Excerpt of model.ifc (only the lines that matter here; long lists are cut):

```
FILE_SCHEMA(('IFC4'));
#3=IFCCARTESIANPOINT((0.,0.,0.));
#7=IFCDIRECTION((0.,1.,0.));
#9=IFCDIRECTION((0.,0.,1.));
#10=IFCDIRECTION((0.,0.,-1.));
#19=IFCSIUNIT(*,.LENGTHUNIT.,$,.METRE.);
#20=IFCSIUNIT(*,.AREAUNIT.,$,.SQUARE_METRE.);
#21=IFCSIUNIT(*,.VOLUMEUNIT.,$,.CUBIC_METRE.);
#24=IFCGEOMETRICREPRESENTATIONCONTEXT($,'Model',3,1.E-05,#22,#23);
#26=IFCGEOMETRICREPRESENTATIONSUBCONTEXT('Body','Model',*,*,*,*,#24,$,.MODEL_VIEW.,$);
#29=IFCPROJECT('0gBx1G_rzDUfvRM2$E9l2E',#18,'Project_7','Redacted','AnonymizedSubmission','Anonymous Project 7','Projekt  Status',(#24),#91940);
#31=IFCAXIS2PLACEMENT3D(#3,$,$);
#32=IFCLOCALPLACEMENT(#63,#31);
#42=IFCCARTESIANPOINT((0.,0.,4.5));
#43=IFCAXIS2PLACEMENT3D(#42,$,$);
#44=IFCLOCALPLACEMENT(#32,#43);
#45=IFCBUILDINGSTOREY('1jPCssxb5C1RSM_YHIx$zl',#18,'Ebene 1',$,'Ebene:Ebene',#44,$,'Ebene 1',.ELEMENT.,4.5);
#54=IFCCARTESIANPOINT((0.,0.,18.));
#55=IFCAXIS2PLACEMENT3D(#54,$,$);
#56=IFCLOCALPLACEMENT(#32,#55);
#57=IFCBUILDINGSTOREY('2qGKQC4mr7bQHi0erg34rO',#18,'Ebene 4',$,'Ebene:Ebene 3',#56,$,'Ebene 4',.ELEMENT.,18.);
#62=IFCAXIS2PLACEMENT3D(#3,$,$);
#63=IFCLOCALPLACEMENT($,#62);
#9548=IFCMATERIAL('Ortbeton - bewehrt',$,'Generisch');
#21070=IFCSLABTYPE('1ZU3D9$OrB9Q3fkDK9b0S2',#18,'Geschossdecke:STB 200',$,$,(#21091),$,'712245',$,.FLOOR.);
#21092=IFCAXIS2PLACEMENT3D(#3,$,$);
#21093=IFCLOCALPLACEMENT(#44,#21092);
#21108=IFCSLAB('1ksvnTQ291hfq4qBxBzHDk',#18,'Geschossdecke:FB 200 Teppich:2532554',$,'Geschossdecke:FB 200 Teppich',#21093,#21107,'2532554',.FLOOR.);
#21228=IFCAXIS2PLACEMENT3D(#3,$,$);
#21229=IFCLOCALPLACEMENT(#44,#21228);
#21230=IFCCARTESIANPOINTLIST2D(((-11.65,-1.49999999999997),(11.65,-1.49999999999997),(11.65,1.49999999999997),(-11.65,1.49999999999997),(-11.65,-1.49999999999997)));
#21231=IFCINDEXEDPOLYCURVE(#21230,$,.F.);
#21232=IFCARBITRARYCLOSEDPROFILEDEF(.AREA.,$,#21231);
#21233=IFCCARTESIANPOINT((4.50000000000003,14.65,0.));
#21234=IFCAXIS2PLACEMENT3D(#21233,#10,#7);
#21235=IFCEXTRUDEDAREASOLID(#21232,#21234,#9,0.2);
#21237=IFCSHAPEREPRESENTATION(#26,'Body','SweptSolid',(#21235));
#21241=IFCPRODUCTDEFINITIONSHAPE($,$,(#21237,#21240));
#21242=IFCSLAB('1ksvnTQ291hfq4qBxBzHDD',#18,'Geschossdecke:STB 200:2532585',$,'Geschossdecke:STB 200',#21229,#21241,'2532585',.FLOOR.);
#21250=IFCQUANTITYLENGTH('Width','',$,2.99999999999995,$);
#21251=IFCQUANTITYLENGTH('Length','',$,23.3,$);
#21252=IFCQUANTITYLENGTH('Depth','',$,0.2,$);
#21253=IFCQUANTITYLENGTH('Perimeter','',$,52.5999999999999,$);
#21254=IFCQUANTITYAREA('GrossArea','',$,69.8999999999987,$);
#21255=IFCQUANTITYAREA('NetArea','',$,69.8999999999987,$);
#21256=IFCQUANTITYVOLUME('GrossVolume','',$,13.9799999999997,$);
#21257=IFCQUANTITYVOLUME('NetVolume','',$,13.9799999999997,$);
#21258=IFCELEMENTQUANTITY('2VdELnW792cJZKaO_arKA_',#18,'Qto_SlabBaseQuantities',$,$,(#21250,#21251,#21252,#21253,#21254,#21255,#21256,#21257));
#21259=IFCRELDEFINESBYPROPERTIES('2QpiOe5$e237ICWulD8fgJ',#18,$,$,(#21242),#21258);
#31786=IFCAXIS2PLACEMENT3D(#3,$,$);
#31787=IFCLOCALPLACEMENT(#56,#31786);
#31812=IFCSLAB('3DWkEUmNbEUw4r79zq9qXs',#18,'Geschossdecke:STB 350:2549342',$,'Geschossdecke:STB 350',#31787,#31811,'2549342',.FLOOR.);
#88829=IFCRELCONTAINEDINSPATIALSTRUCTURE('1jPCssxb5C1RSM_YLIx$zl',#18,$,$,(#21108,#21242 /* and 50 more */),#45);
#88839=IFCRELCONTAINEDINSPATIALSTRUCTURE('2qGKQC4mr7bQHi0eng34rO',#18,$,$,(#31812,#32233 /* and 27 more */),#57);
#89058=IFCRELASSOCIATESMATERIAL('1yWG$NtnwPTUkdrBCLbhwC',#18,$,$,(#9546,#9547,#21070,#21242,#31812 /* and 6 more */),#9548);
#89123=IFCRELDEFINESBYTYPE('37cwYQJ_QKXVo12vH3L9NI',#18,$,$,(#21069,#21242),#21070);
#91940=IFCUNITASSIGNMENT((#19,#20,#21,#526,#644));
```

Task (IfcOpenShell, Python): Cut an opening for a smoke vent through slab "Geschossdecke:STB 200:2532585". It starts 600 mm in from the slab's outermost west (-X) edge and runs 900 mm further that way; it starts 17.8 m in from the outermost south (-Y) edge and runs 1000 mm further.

```python
import numpy as np
import ifcopenshell
import ifcopenshell.api.feature
import ifcopenshell.api.geometry
import ifcopenshell.api.pset
import ifcopenshell.api.root
import ifcopenshell.geom
import ifcopenshell.util.element
import ifcopenshell.util.placement
import ifcopenshell.util.representation
import ifcopenshell.util.shape
import ifcopenshell.util.unit

model = ifcopenshell.open("model.ifc")
unit_scale = ifcopenshell.util.unit.calculate_unit_scale(model)
area_scale = ifcopenshell.util.unit.calculate_unit_scale(model, "AREAUNIT")
volume_scale = ifcopenshell.util.unit.calculate_unit_scale(model, "VOLUMEUNIT")
settings = ifcopenshell.geom.settings()


def volume(element):
    """Net volume in cubic metres, openings subtracted."""
    shape = ifcopenshell.geom.create_shape(settings, element)
    return ifcopenshell.util.shape.get_volume(shape.geometry)


slab = model.by_id(21242)
before = volume(slab)

# Extent in the slab's own axes, in metres. The edges named are its -X and -Y sides.
slab_shape = ifcopenshell.geom.create_shape(settings, slab)
vertices = ifcopenshell.util.shape.get_vertices(slab_shape.geometry)
x_min, y_min, bottom = vertices.min(axis=0)
top = vertices[:, 2].max()

opening = ifcopenshell.api.root.create_entity(model, ifc_class="IfcOpeningElement", name="Smoke vent opening", predefined_type="OPENING")
context = ifcopenshell.util.representation.get_context(model, "Model", "Body", "MODEL_VIEW")
width, depth = 0.9, 1
outline = [(0.0, 0.0), (width, 0.0), (width, depth), (0.0, depth), (0.0, 0.0)]
# Overshoot both faces by 50 mm so the cut is clean.
shape = ifcopenshell.api.geometry.add_slab_representation(
    model, context=context, depth=top - bottom + 0.1, polyline=outline
)
ifcopenshell.api.geometry.assign_representation(model, product=opening, representation=shape)

matrix = ifcopenshell.util.placement.get_local_placement(slab.ObjectPlacement)
matrix[:, 3] = matrix @ np.append(np.array([x_min + 0.6, y_min + 17.8, bottom - 0.05]) / unit_scale, 1.0)
ifcopenshell.api.geometry.edit_object_placement(model, product=opening, matrix=matrix, is_si=False)
ifcopenshell.api.feature.add_feature(model, feature=opening, element=slab)

after = volume(slab)

# Update the slab's stored quantities.
qto = model.by_id(ifcopenshell.util.element.get_pset(slab, "Qto_SlabBaseQuantities", should_inherit=False)["id"])
ifcopenshell.api.pset.edit_qto(model, qto=qto, properties={
    "NetArea": after / (top - bottom) / area_scale,
    "NetVolume": after / volume_scale,
})

print(f"slab volume {before:.3f} -> {after:.3f} m3")

model.write("model_updated.ifc")
```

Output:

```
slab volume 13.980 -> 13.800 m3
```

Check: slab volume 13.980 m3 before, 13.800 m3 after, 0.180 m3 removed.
